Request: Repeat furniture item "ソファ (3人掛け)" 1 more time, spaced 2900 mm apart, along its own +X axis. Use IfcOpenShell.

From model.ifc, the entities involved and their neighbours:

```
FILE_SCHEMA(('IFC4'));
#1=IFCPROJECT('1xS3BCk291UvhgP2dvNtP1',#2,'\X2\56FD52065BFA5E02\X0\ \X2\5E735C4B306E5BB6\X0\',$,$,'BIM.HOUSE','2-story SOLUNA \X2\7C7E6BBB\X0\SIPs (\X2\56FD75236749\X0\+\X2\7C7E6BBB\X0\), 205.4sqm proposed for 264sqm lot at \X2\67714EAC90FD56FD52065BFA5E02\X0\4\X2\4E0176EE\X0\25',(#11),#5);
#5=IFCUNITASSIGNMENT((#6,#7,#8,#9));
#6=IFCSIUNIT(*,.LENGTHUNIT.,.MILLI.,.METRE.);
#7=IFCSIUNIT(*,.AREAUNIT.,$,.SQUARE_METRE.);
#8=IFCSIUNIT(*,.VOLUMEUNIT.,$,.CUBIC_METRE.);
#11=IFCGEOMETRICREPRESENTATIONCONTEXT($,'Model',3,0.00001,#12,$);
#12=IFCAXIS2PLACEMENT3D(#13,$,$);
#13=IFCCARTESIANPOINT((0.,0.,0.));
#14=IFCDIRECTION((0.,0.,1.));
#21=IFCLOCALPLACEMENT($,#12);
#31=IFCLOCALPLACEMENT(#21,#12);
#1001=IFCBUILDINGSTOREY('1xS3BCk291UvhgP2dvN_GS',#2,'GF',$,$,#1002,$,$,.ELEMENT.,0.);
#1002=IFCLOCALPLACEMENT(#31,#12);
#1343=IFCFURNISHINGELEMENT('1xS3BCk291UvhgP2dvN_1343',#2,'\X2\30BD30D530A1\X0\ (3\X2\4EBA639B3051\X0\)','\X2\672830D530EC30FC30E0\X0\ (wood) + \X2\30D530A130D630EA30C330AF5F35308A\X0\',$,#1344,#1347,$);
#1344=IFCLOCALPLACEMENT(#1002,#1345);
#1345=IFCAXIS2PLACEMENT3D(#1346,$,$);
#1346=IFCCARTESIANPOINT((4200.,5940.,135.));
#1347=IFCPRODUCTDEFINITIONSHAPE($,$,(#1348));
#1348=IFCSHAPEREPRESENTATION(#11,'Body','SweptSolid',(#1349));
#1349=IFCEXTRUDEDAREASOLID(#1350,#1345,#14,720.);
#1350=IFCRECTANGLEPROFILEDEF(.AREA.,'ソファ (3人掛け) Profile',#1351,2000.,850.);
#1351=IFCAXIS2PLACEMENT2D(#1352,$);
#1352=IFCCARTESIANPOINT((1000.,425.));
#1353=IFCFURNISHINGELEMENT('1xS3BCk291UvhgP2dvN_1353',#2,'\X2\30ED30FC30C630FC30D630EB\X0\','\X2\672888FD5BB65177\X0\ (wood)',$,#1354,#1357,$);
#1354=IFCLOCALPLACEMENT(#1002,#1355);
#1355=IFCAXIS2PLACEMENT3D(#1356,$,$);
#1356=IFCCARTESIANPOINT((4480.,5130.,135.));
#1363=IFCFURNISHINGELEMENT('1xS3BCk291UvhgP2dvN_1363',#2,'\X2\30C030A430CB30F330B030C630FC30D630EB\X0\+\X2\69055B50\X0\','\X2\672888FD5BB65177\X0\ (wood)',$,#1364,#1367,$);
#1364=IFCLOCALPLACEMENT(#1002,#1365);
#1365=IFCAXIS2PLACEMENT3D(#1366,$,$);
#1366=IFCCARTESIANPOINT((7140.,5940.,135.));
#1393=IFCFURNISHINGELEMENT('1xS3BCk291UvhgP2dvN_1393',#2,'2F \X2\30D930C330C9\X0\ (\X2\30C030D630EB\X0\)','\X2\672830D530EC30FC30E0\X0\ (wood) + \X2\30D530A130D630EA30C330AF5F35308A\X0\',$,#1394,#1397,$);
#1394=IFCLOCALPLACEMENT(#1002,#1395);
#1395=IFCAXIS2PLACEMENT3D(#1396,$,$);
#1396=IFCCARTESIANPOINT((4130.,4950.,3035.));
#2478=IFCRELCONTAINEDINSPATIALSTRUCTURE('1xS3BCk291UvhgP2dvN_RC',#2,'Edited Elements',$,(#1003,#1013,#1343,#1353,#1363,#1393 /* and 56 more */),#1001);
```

```python
import ifcopenshell
import ifcopenshell.api.geometry
import ifcopenshell.api.root
import ifcopenshell.util.element
import ifcopenshell.util.placement
import ifcopenshell.util.unit

model = ifcopenshell.open("model.ifc")
unit_scale = ifcopenshell.util.unit.calculate_unit_scale(model)


def reuse_history(source, copy):
    """copy_class also copies each property set's owner history, people and application; keep the originals."""
    for rel in copy.IsDefinedBy:
        if rel.is_a("IfcRelDefinesByProperties") and (history := rel.RelatingPropertyDefinition.OwnerHistory):
            rel.RelatingPropertyDefinition.OwnerHistory = source.OwnerHistory
            ifcopenshell.util.element.remove_deep2(model, history)


source = model.by_id(1343)
base = ifcopenshell.util.placement.get_local_placement(source.ObjectPlacement)
step = base[:3, 0] * 2.9 / unit_scale

for i in range(1, 2):
    copy = ifcopenshell.api.root.copy_class(model, product=source)
    copy.Representation = ifcopenshell.util.element.copy_deep(
        model, source.Representation, exclude=["IfcGeometricRepresentationContext", "IfcRepresentationMap"]
    )
    reuse_history(source, copy)
    matrix = base.copy()
    matrix[:3, 3] += i * step
    print("added at", matrix[:3, 3].round(3) + 0.0)
    ifcopenshell.api.geometry.edit_object_placement(model, product=copy, matrix=matrix, is_si=False)

model.write("model_edited.ifc")
```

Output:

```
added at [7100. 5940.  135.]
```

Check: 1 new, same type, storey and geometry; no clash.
